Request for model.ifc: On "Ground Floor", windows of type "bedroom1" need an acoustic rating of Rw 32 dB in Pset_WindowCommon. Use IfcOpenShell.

First a look at what the model holds.

```python
import ifcopenshell
import ifcopenshell.util.element

model = ifcopenshell.open("model.ifc")
print(model.schema)
storey = next(s for s in model.by_type("IfcBuildingStorey") if s.Name == "Ground Floor")
windows = [e for e in ifcopenshell.util.element.get_decomposition(storey) if e.is_a("IfcWindow")]
seen = {}
for e in windows:
    element_type = ifcopenshell.util.element.get_type(e)
    key = (element_type.Name if element_type != e and element_type else None, ifcopenshell.util.element.get_pset(e, "Pset_WindowCommon", "AcousticRating"))
    seen[key] = seen.get(key, 0) + 1
for (name, value), count in sorted(seen.items(), key=str):
    print(count, "x", name, "|", value)
```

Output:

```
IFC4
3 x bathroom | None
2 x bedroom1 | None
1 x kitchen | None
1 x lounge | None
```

```python
import ifcopenshell
import ifcopenshell.api.pset
import ifcopenshell.util.element

model = ifcopenshell.open("model.ifc")

storey = next(s for s in model.by_type("IfcBuildingStorey") if s.Name == "Ground Floor")
windows = [e for e in ifcopenshell.util.element.get_decomposition(storey) if e.is_a("IfcWindow")]

count = 0
for e in windows:
    element_type = ifcopenshell.util.element.get_type(e)
    if element_type in (None, e) or element_type.Name != "bedroom1":
        continue
    # add_pset returns the element's existing set when there is one.
    pset = ifcopenshell.api.pset.add_pset(model, product=e, name="Pset_WindowCommon")
    ifcopenshell.api.pset.edit_pset(model, pset=pset, properties={"AcousticRating": "Rw 32 dB"})
    count += 1

print(count, "windows updated")

model.write("model_v2.ifc")
```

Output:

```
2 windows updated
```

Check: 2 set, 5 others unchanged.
